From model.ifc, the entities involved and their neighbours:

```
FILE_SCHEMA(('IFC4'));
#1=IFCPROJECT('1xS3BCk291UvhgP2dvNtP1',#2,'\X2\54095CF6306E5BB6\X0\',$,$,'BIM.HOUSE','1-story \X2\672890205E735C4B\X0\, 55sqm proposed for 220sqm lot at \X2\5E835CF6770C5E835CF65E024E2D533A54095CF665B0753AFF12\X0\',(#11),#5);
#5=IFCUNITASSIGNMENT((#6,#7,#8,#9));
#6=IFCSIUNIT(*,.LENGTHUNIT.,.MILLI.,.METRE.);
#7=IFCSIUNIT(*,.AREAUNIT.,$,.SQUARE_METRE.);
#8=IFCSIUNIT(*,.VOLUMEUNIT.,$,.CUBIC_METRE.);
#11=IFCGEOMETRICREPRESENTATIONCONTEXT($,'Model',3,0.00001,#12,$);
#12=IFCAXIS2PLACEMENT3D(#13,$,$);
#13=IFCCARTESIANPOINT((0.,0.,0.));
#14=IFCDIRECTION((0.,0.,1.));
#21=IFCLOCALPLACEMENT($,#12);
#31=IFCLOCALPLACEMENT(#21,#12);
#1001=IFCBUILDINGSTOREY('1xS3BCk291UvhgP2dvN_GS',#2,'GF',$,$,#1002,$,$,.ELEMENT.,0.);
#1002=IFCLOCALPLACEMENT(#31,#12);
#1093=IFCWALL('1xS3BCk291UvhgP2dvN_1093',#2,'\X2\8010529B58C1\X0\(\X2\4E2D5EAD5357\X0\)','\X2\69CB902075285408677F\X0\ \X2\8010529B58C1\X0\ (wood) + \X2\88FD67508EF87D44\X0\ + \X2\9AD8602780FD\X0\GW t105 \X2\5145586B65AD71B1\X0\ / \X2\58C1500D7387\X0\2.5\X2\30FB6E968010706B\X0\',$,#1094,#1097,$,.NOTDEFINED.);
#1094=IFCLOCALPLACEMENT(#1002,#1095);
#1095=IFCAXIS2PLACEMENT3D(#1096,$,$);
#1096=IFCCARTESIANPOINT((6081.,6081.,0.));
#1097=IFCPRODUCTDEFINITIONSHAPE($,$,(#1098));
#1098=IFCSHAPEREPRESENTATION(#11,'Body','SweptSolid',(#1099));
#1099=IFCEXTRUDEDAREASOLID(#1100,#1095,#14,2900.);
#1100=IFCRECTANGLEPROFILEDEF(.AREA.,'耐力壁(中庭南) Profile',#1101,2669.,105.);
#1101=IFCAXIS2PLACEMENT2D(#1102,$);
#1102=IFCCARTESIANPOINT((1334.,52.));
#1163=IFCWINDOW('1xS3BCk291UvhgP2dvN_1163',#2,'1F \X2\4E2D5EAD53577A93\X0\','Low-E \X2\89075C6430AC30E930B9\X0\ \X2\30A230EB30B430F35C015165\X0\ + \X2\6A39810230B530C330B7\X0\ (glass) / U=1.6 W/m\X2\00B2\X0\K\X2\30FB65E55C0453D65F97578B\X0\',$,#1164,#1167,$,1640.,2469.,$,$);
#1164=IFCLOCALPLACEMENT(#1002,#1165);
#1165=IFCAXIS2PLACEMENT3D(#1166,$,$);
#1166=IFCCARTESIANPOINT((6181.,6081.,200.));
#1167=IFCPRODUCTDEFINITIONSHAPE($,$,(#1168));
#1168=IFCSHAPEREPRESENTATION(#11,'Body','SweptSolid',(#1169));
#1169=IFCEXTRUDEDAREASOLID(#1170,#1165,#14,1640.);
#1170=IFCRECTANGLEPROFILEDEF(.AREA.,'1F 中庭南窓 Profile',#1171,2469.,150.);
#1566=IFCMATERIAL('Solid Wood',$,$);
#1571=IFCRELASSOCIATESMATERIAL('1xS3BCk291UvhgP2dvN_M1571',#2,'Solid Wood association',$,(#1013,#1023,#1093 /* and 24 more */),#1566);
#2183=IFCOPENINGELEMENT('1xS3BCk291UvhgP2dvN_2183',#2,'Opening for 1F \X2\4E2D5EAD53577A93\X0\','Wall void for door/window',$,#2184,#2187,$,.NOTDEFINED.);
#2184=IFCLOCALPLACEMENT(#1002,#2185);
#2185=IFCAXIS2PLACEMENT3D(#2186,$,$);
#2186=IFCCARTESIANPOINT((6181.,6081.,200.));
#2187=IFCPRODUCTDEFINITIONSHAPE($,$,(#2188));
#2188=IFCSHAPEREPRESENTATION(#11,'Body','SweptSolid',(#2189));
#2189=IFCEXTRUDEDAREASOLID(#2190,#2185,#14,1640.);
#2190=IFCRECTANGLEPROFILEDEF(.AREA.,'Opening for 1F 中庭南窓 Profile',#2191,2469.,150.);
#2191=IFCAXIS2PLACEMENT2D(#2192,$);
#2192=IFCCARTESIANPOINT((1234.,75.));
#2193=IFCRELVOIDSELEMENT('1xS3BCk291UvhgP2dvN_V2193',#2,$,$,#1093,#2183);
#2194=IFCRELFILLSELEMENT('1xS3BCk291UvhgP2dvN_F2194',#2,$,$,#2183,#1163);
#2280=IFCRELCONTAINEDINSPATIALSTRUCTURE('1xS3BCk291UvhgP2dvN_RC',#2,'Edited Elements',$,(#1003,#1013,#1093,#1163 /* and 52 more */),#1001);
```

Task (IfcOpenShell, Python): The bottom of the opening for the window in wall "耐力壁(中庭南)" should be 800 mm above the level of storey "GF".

```python
import numpy as np
import ifcopenshell
import ifcopenshell.api.geometry
import ifcopenshell.geom
import ifcopenshell.util.element
import ifcopenshell.util.placement
import ifcopenshell.util.shape
import ifcopenshell.util.unit

model = ifcopenshell.open("model.ifc")
unit_scale = ifcopenshell.util.unit.calculate_unit_scale(model)

window = model.by_id(1163)
opening = window.FillsVoids[0].RelatingOpeningElement
storey = ifcopenshell.util.element.get_container(window, ifc_class="IfcBuildingStorey")
level = ifcopenshell.util.placement.get_local_placement(storey.ObjectPlacement)[2, 3]

# The opening's origin need not be at the sill, so measure its lowest point.
shape = ifcopenshell.geom.create_shape(ifcopenshell.geom.settings(), opening)
bottom = ifcopenshell.util.shape.get_shape_bottom_elevation(shape, shape.geometry) / unit_scale
dz = level + 800.0 - bottom

shift = np.array([0.0, 0.0, dz])
# The window is not placed relative to its opening, so move both.
for product in (opening, window):
    matrix = ifcopenshell.util.placement.get_local_placement(product.ObjectPlacement)
    matrix[:3, 3] += shift
    ifcopenshell.api.geometry.edit_object_placement(model, product=product, matrix=matrix, is_si=False)

print(f"moved by {dz * unit_scale:+.3f} m")

model.write("model-out.ifc")
```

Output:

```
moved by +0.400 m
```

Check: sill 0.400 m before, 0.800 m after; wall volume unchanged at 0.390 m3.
